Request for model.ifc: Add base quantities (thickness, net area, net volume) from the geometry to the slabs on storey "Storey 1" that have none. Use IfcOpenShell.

First a look at what the model holds.

```python
import ifcopenshell
import ifcopenshell.util.element
import ifcopenshell.util.unit

model = ifcopenshell.open("model.ifc")
print(model.schema)
for unit_type in ("LENGTHUNIT", "AREAUNIT", "VOLUMEUNIT"):
    print(unit_type, ifcopenshell.util.unit.calculate_unit_scale(model, unit_type))
storey = next(s for s in model.by_type("IfcBuildingStorey") if s.Name == "Storey 1")
slabs = [e for e in ifcopenshell.util.element.get_decomposition(storey) if e.is_a("IfcSlab")]
for e in sorted(slabs, key=lambda e: e.id()):
    print(e.id(), e.is_a(), e.Name, list(ifcopenshell.util.element.get_psets(e, qtos_only=True)), sep=" | ")
```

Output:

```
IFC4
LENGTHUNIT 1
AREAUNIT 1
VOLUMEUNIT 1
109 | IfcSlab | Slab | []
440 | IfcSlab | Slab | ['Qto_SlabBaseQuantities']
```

```python
import ifcopenshell
import ifcopenshell.api.pset
import ifcopenshell.geom
import ifcopenshell.util.element
import ifcopenshell.util.shape
import ifcopenshell.util.unit

model = ifcopenshell.open("model.ifc")
unit_scale = ifcopenshell.util.unit.calculate_unit_scale(model)
area_scale = ifcopenshell.util.unit.calculate_unit_scale(model, "AREAUNIT")
volume_scale = ifcopenshell.util.unit.calculate_unit_scale(model, "VOLUMEUNIT")
settings = ifcopenshell.geom.settings()

storey = next(s for s in model.by_type("IfcBuildingStorey") if s.Name == "Storey 1")
slabs = [e for e in ifcopenshell.util.element.get_decomposition(storey) if e.is_a("IfcSlab")]

for e in sorted(slabs, key=lambda e: e.id()):
    if ifcopenshell.util.element.get_psets(e, qtos_only=True, should_inherit=False):
        continue
    # Geometry comes back in metres, in the element's own axes.
    shape = ifcopenshell.geom.create_shape(settings, e)
    values = {
        "Width": ifcopenshell.util.shape.get_z(shape.geometry) / unit_scale,
        "NetArea": ifcopenshell.util.shape.get_footprint_area(shape.geometry) / area_scale,
        "NetVolume": ifcopenshell.util.shape.get_volume(shape.geometry) / volume_scale,
    }
    qto = ifcopenshell.api.pset.add_qto(model, product=e, name="Qto_SlabBaseQuantities")
    ifcopenshell.api.pset.edit_qto(model, qto=qto, properties=values)
    print(e.id(), {k: round(v, 3) for k, v in values.items()})

model.write("model_updated.ifc")
```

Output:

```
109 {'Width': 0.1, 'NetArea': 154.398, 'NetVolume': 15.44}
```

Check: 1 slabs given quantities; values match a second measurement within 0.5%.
